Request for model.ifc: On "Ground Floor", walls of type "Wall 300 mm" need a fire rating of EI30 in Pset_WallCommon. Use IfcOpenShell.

First a look at what the model holds.

```python
import ifcopenshell
import ifcopenshell.util.element

model = ifcopenshell.open("model.ifc")
print(model.schema)
storey = next(s for s in model.by_type("IfcBuildingStorey") if s.Name == "Ground Floor")
walls = [e for e in ifcopenshell.util.element.get_decomposition(storey) if e.is_a("IfcWall")]
seen = {}
for e in walls:
    element_type = ifcopenshell.util.element.get_type(e)
    key = (element_type.Name if element_type != e and element_type else None, ifcopenshell.util.element.get_pset(e, "Pset_WallCommon", "FireRating"))
    seen[key] = seen.get(key, 0) + 1
for (name, value), count in sorted(seen.items(), key=str):
    print(count, "x", name, "|", value)
```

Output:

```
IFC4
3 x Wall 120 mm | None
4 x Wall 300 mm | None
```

```python
import ifcopenshell
import ifcopenshell.api.pset
import ifcopenshell.util.element

model = ifcopenshell.open("model.ifc")

storey = next(s for s in model.by_type("IfcBuildingStorey") if s.Name == "Ground Floor")
walls = [e for e in ifcopenshell.util.element.get_decomposition(storey) if e.is_a("IfcWall")]

count = 0
for e in walls:
    element_type = ifcopenshell.util.element.get_type(e)
    if element_type in (None, e) or element_type.Name != "Wall 300 mm":
        continue
    # add_pset returns the element's existing set when there is one.
    pset = ifcopenshell.api.pset.add_pset(model, product=e, name="Pset_WallCommon")
    ifcopenshell.api.pset.edit_pset(model, pset=pset, properties={"FireRating": "EI30"})
    count += 1

print(count, "walls updated")

model.write("model_edited.ifc")
```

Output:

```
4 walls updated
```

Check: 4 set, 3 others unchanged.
